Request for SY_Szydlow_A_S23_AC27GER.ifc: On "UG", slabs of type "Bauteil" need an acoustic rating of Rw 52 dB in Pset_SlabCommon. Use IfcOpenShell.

First a look at what the model holds.

```python
import ifcopenshell
import ifcopenshell.util.element

model = ifcopenshell.open("SY_Szydlow_A_S23_AC27GER.ifc")
print(model.schema)
storey = next(s for s in model.by_type("IfcBuildingStorey") if s.Name == "UG")
slabs = [e for e in ifcopenshell.util.element.get_decomposition(storey) if e.is_a("IfcSlab")]
seen = {}
for e in slabs:
    element_type = ifcopenshell.util.element.get_type(e)
    key = (element_type.Name if element_type != e and element_type else None, ifcopenshell.util.element.get_pset(e, "Pset_SlabCommon", "AcousticRating"))
    seen[key] = seen.get(key, 0) + 1
for (name, value), count in sorted(seen.items(), key=str):
    print(count, "x", name, "|", value)
```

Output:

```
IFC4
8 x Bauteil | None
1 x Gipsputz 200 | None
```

```python
import ifcopenshell
import ifcopenshell.api.pset
import ifcopenshell.util.element

model = ifcopenshell.open("SY_Szydlow_A_S23_AC27GER.ifc")

storey = next(s for s in model.by_type("IfcBuildingStorey") if s.Name == "UG")
slabs = [e for e in ifcopenshell.util.element.get_decomposition(storey) if e.is_a("IfcSlab")]

count = 0
for e in slabs:
    element_type = ifcopenshell.util.element.get_type(e)
    if element_type in (None, e) or element_type.Name != "Bauteil":
        continue
    # add_pset returns the element's existing set when there is one.
    pset = ifcopenshell.api.pset.add_pset(model, product=e, name="Pset_SlabCommon")
    ifcopenshell.api.pset.edit_pset(model, pset=pset, properties={"AcousticRating": "Rw 52 dB"})
    count += 1

print(count, "slabs updated")

model.write("SY_Szydlow_A_S23_AC27GER_rev.ifc")
```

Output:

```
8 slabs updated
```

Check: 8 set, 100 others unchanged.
